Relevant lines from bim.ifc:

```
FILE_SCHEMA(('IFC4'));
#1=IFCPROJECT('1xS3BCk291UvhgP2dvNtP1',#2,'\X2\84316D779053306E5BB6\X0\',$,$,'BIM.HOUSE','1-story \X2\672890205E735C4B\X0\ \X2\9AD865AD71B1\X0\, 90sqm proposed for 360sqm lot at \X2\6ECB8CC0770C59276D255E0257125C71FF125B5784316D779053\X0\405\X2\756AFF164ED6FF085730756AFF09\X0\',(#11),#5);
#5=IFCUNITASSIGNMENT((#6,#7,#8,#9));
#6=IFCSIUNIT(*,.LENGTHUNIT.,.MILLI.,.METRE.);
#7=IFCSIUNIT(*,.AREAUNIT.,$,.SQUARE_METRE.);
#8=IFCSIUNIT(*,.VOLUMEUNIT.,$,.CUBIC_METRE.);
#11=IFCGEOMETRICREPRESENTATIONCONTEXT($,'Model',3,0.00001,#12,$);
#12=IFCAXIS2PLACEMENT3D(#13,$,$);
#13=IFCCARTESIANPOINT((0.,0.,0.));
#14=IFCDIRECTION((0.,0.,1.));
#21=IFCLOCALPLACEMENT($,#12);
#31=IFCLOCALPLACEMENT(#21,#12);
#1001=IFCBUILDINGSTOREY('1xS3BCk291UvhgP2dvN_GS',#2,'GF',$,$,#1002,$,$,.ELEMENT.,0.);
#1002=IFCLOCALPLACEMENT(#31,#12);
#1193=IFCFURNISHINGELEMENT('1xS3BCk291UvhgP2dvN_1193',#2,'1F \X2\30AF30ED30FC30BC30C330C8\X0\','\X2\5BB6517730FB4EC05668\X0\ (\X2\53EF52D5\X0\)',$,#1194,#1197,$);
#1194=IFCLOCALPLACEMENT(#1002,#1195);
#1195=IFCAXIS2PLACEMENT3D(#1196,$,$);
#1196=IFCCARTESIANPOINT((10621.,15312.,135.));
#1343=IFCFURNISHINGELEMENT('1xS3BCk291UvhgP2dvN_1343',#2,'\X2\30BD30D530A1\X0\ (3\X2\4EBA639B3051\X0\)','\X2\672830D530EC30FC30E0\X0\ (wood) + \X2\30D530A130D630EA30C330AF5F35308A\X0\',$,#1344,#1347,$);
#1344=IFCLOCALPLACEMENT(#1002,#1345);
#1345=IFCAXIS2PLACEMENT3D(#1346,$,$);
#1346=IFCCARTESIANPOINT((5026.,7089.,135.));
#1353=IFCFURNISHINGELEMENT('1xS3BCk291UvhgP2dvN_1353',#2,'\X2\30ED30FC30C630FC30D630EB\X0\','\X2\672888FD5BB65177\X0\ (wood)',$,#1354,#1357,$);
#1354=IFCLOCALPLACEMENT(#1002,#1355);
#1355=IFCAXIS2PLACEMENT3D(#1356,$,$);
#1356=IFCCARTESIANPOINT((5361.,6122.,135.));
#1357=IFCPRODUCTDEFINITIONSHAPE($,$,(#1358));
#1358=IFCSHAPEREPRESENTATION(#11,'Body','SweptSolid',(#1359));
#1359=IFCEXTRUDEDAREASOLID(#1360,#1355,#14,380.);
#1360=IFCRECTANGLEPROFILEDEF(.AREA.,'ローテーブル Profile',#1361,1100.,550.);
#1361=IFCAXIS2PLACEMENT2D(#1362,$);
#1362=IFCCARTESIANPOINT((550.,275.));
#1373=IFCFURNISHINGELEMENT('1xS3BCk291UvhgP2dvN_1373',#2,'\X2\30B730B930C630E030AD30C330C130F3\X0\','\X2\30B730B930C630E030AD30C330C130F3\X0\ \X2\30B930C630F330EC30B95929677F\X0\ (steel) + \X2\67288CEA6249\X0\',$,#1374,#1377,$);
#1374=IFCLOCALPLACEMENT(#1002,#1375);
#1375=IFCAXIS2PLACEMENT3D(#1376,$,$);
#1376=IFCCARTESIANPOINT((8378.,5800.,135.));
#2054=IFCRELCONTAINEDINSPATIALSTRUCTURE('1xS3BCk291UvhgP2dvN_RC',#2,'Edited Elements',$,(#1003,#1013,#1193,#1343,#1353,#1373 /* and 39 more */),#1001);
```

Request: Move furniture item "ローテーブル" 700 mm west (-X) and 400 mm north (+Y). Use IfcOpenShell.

```python
import ifcopenshell
import ifcopenshell.api.geometry
import ifcopenshell.util.placement

model = ifcopenshell.open("bim.ifc")

item = model.by_guid("1xS3BCk291UvhgP2dvN_1353")
matrix = ifcopenshell.util.placement.get_local_placement(item.ObjectPlacement)
matrix[0, 3] -= 700.0
matrix[1, 3] += 400.0
ifcopenshell.api.geometry.edit_object_placement(model, product=item, matrix=matrix, is_si=False)

print(ifcopenshell.util.placement.get_local_placement(item.ObjectPlacement).round(3) + 0.0)

model.write("bim_edited.ifc")
```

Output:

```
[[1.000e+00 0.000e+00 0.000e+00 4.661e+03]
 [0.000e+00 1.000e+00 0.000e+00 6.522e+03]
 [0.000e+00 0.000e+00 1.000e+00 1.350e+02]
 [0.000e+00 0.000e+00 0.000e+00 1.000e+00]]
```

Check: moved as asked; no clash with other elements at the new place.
